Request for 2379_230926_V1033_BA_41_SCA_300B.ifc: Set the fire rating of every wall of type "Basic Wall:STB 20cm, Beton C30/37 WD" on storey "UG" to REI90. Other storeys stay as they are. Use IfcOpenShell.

First a look at what the model holds.

```python
import ifcopenshell
import ifcopenshell.util.element

model = ifcopenshell.open("2379_230926_V1033_BA_41_SCA_300B.ifc")
print(model.schema)
storey = next(s for s in model.by_type("IfcBuildingStorey") if s.Name == "UG")
walls = [e for e in ifcopenshell.util.element.get_decomposition(storey) if e.is_a("IfcWall")]
seen = {}
for e in walls:
    element_type = ifcopenshell.util.element.get_type(e)
    key = (element_type.Name if element_type != e and element_type else None, ifcopenshell.util.element.get_pset(e, "Pset_WallCommon", "FireRating"))
    seen[key] = seen.get(key, 0) + 1
for (name, value), count in sorted(seen.items(), key=str):
    print(count, "x", name, "|", value)
```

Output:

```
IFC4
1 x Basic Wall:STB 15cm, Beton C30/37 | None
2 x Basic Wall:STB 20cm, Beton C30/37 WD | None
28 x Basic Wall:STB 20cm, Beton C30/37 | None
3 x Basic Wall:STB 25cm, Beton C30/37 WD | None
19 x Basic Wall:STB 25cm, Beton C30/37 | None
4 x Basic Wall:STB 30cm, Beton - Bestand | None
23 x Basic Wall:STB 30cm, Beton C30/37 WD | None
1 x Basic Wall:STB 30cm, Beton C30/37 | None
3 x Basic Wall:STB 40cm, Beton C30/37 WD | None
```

```python
import ifcopenshell
import ifcopenshell.api.pset
import ifcopenshell.util.element

model = ifcopenshell.open("2379_230926_V1033_BA_41_SCA_300B.ifc")

storey = next(s for s in model.by_type("IfcBuildingStorey") if s.Name == "UG")
walls = [e for e in ifcopenshell.util.element.get_decomposition(storey) if e.is_a("IfcWall")]

count = 0
for e in walls:
    element_type = ifcopenshell.util.element.get_type(e)
    if element_type in (None, e) or element_type.Name != "Basic Wall:STB 20cm, Beton C30/37 WD":
        continue
    # add_pset returns the element's existing set when there is one.
    pset = ifcopenshell.api.pset.add_pset(model, product=e, name="Pset_WallCommon")
    ifcopenshell.api.pset.edit_pset(model, pset=pset, properties={"FireRating": "REI90"})
    count += 1

print(count, "walls updated")

model.write("2379_230926_V1033_BA_41_SCA_300B_updated.ifc")
```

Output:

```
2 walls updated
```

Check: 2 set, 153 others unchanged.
